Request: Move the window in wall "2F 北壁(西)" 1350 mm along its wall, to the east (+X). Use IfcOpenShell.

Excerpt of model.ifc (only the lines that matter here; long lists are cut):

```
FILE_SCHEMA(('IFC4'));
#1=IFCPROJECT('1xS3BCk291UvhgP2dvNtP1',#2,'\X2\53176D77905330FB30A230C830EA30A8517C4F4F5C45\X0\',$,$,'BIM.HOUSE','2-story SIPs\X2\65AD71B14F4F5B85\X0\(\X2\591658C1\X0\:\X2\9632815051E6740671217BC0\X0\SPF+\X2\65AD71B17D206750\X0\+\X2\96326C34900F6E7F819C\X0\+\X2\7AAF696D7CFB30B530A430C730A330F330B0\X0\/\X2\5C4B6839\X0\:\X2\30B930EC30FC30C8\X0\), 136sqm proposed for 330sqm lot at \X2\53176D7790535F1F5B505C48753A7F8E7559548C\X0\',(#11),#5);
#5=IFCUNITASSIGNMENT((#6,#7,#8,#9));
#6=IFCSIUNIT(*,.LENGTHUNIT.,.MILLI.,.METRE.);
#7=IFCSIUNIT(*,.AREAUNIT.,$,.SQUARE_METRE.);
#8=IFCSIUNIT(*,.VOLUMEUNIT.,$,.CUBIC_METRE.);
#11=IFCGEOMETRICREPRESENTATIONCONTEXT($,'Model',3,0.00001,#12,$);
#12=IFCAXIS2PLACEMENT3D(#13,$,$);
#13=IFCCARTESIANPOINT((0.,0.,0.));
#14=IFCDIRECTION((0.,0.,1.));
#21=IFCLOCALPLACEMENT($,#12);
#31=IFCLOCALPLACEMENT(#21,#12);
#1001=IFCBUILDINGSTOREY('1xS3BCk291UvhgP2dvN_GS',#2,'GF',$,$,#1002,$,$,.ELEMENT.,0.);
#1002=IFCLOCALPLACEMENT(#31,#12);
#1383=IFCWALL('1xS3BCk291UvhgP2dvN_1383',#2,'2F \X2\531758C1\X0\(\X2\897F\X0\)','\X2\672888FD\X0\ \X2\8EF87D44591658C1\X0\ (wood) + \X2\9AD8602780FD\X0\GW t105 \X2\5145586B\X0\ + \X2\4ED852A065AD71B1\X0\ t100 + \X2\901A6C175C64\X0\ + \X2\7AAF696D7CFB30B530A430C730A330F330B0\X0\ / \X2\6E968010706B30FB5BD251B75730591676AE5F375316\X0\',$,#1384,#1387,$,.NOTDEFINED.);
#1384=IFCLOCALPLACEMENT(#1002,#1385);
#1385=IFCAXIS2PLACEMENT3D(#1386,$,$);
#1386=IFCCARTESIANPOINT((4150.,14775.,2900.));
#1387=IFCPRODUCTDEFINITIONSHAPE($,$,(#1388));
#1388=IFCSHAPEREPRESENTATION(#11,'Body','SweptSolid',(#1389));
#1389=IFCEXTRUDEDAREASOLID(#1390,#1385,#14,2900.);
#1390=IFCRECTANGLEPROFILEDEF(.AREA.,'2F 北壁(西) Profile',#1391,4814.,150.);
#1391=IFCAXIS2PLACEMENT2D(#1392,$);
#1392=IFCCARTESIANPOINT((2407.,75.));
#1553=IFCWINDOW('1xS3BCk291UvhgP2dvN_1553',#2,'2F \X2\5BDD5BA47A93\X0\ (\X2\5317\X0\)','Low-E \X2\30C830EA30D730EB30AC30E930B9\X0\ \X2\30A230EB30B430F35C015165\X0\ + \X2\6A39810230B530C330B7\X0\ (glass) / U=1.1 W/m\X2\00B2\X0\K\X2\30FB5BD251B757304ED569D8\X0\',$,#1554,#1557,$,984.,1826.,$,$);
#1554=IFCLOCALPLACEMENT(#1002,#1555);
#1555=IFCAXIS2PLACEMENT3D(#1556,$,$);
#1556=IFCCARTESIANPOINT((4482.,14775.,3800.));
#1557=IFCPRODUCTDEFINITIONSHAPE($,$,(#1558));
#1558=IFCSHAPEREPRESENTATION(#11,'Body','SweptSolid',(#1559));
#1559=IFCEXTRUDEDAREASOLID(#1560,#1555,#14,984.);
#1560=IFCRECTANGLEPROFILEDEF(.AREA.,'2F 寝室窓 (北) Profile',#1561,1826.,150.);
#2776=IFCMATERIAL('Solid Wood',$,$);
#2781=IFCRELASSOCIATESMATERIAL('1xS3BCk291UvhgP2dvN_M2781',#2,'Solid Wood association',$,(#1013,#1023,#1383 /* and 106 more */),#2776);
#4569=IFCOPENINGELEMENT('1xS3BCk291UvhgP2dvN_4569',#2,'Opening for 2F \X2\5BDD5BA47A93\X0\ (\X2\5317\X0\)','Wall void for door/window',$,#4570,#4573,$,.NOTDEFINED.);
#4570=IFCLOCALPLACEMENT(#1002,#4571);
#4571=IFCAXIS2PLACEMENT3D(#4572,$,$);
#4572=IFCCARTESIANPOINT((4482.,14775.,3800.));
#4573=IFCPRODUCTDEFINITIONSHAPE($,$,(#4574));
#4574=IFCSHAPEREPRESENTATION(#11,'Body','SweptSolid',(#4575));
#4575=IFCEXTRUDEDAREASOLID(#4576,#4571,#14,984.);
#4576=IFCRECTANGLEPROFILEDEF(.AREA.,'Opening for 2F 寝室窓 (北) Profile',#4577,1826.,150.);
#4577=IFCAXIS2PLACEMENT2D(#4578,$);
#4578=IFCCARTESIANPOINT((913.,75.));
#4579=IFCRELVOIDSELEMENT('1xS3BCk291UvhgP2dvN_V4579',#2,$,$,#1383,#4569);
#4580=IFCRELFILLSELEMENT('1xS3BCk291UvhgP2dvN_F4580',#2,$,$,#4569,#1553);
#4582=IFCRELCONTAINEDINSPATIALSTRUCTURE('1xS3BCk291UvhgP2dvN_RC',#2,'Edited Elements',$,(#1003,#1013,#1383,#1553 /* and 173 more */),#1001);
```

```python
import ifcopenshell
import ifcopenshell.api.geometry
import ifcopenshell.util.placement
import ifcopenshell.util.unit

model = ifcopenshell.open("model.ifc")
unit_scale = ifcopenshell.util.unit.calculate_unit_scale(model)

window = model.by_guid("1xS3BCk291UvhgP2dvN_1553")
opening = window.FillsVoids[0].RelatingOpeningElement
wall = opening.VoidsElements[0].RelatingBuildingElement

wall_matrix = ifcopenshell.util.placement.get_local_placement(wall.ObjectPlacement)
shift = wall_matrix[:3, 0] * 1.35 / unit_scale
before = ifcopenshell.util.placement.get_local_placement(window.ObjectPlacement)[:3, 3].copy()

# The window is not placed relative to its opening, so move both.
for product in (opening, window):
    matrix = ifcopenshell.util.placement.get_local_placement(product.ObjectPlacement)
    matrix[:3, 3] += shift
    ifcopenshell.api.geometry.edit_object_placement(model, product=product, matrix=matrix, is_si=False)

after = ifcopenshell.util.placement.get_local_placement(window.ObjectPlacement)[:3, 3]
print("window moved by", (after - before).round(3) + 0.0)

model.write("model_edited.ifc")
```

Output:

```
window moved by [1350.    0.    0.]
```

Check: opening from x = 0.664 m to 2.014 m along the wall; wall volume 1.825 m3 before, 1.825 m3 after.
